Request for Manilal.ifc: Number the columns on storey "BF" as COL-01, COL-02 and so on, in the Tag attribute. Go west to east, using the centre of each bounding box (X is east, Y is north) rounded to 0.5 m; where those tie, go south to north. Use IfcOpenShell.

First a look at what the model holds.

```python
import ifcopenshell
import ifcopenshell.util.element
import ifcopenshell.util.placement

model = ifcopenshell.open("Manilal.ifc")
print(model.schema)
storey = next(s for s in model.by_type("IfcBuildingStorey") if s.Name == "BF")
columns = [e for e in ifcopenshell.util.element.get_decomposition(storey) if e.is_a("IfcColumn")]
for e in sorted(columns, key=lambda e: e.id()):
    origin = ifcopenshell.util.placement.get_local_placement(e.ObjectPlacement)[:3, 3]
    print(e.id(), e.Tag, e.Name, origin.round(2) + 0.0, sep=" | ")
```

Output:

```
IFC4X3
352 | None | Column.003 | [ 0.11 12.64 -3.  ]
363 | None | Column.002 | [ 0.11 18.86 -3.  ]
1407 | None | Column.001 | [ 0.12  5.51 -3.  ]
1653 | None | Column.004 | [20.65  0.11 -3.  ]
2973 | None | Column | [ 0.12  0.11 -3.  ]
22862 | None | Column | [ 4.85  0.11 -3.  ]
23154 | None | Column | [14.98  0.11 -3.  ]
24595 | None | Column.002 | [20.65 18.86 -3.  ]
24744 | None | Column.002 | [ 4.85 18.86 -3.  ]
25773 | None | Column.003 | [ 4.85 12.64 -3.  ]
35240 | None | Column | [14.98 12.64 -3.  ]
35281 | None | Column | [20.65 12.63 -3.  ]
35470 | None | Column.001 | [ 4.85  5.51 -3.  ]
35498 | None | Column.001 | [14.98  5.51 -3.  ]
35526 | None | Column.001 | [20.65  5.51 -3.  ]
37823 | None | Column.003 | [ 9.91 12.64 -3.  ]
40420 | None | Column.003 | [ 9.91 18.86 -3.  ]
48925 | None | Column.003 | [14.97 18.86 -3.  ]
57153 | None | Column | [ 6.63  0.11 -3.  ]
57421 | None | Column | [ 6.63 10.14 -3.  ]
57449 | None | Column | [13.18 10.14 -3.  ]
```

```python
import ifcopenshell
import ifcopenshell.geom
import ifcopenshell.util.element
import ifcopenshell.util.shape

model = ifcopenshell.open("Manilal.ifc")
settings = ifcopenshell.geom.settings()
settings.set("use-world-coords", True)


def centre(element):
    shape = ifcopenshell.geom.create_shape(settings, element)
    return ifcopenshell.util.shape.get_bbox_centroid(shape.geometry)


storey = next(s for s in model.by_type("IfcBuildingStorey") if s.Name == "BF")
columns = [e for e in ifcopenshell.util.element.get_decomposition(storey) if e.is_a("IfcColumn")]

# Insertion points can sit at a corner or the storey origin, so sort by the geometry (in metres).
centres = {e: centre(e) for e in columns}
columns.sort(key=lambda e: (round(centres[e][0] / 0.5), centres[e][1]))

for i, e in enumerate(columns, start=1):
    number = f"COL-{i:02d}"
    e.Tag = number
    print(e.id(), number)

model.write("Manilal_rev.ifc")
```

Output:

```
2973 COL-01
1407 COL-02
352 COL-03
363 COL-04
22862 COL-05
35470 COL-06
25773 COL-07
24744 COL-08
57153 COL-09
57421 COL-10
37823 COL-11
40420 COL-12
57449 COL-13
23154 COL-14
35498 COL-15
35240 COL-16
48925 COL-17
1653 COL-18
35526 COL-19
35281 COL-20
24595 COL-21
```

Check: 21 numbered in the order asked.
